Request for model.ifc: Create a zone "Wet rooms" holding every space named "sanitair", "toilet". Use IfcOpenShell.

First a look at what the model holds.

```python
import ifcopenshell

model = ifcopenshell.open("model.ifc")
print(model.schema)
seen = {}
for space in model.by_type("IfcSpace"):
    seen[space.LongName] = seen.get(space.LongName, 0) + 1
for name, count in sorted(seen.items(), key=str):
    print(count, "x", name)
print("zones:", [z.Name for z in model.by_type("IfcZone")][:20])
```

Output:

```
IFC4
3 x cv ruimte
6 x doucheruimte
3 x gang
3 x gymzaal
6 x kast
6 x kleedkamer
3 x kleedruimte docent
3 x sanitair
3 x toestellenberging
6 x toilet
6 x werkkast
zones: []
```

```python
import ifcopenshell
import ifcopenshell.api.group
import ifcopenshell.api.root

model = ifcopenshell.open("model.ifc")

names = {"sanitair", "toilet"}
spaces = [s for s in model.by_type("IfcSpace") if s.LongName in names]

zone = ifcopenshell.api.root.create_entity(model, ifc_class="IfcZone", name="Wet rooms")
ifcopenshell.api.group.assign_group(model, products=spaces, group=zone)
print(len(spaces), "spaces in", zone.Name)

model.write("model_rev.ifc")
```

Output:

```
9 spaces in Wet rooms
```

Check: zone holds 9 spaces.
